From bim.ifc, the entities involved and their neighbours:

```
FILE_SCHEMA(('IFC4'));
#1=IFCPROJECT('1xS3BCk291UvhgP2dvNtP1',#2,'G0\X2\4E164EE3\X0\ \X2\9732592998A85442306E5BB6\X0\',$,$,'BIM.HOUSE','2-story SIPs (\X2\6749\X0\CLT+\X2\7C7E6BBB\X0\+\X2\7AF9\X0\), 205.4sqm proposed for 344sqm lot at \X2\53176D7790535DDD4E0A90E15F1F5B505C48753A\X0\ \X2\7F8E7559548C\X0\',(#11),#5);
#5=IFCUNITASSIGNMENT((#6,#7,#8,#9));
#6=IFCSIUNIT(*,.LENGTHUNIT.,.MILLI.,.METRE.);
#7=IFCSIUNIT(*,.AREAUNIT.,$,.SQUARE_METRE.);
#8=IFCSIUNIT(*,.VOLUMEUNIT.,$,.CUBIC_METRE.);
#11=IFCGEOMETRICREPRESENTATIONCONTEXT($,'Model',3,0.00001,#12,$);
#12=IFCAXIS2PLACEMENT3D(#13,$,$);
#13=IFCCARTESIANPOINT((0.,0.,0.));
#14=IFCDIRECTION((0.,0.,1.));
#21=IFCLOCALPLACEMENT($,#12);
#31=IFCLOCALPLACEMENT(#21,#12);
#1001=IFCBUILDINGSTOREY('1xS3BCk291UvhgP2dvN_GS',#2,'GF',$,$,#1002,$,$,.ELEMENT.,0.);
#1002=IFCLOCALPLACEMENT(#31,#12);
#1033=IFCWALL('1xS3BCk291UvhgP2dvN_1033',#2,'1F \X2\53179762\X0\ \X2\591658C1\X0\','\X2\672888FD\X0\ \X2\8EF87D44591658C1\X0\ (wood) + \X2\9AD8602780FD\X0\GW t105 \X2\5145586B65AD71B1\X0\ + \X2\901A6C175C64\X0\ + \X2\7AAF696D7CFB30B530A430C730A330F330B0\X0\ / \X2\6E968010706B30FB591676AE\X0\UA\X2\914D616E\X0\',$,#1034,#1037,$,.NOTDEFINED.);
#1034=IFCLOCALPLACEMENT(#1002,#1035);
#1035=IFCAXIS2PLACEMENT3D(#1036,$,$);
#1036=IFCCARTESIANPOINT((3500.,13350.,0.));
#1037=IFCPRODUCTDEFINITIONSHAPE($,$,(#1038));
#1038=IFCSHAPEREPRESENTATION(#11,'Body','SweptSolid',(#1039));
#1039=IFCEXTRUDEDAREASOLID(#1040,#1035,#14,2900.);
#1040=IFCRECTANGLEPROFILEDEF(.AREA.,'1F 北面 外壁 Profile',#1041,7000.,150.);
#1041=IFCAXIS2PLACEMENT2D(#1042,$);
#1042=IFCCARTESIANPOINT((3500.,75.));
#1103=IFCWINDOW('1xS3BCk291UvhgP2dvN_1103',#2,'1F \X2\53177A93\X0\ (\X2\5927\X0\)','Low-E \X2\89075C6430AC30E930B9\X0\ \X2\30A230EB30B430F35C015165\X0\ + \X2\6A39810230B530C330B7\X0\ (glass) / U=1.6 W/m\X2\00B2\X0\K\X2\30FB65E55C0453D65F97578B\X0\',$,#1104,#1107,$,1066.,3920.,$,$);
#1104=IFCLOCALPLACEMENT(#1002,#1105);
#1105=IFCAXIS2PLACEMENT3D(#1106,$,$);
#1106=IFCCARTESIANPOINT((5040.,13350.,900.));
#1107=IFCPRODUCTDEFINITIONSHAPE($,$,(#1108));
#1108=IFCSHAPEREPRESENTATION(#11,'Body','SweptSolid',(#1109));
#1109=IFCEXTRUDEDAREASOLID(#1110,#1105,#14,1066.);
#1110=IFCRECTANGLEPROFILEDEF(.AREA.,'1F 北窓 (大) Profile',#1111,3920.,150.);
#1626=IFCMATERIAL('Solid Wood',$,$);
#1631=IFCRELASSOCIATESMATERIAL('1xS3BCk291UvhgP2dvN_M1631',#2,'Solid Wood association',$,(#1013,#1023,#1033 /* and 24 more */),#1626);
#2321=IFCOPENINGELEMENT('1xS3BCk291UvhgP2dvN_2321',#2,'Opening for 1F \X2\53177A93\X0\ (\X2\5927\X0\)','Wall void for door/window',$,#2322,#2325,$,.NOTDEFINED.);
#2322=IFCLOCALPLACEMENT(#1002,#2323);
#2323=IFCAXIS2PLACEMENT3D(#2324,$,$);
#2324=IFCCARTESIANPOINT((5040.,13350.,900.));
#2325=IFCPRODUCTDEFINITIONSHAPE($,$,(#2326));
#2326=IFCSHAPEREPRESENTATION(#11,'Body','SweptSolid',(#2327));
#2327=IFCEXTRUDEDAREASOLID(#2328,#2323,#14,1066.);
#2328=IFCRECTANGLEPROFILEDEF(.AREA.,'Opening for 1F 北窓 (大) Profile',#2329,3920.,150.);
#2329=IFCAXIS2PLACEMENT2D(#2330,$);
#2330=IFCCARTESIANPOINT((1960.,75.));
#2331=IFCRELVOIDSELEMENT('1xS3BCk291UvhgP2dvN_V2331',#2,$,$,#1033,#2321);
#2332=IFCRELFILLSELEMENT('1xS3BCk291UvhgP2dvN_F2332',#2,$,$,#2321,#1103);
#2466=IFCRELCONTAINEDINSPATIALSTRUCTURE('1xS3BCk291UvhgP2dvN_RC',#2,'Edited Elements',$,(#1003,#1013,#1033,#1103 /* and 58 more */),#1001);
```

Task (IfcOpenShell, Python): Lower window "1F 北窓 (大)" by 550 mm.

```python
import numpy as np
import ifcopenshell
import ifcopenshell.api.geometry
import ifcopenshell.util.placement
import ifcopenshell.util.unit

model = ifcopenshell.open("bim.ifc")
unit_scale = ifcopenshell.util.unit.calculate_unit_scale(model)

window = model.by_guid("1xS3BCk291UvhgP2dvN_1103")
opening = window.FillsVoids[0].RelatingOpeningElement
dz = -550.0

shift = np.array([0.0, 0.0, dz])
# The window is not placed relative to its opening, so move both.
for product in (opening, window):
    matrix = ifcopenshell.util.placement.get_local_placement(product.ObjectPlacement)
    matrix[:3, 3] += shift
    ifcopenshell.api.geometry.edit_object_placement(model, product=product, matrix=matrix, is_si=False)

print(f"moved by {dz * unit_scale:+.3f} m")

model.write("bim_updated.ifc")
```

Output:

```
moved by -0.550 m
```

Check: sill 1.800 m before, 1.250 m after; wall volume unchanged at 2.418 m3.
